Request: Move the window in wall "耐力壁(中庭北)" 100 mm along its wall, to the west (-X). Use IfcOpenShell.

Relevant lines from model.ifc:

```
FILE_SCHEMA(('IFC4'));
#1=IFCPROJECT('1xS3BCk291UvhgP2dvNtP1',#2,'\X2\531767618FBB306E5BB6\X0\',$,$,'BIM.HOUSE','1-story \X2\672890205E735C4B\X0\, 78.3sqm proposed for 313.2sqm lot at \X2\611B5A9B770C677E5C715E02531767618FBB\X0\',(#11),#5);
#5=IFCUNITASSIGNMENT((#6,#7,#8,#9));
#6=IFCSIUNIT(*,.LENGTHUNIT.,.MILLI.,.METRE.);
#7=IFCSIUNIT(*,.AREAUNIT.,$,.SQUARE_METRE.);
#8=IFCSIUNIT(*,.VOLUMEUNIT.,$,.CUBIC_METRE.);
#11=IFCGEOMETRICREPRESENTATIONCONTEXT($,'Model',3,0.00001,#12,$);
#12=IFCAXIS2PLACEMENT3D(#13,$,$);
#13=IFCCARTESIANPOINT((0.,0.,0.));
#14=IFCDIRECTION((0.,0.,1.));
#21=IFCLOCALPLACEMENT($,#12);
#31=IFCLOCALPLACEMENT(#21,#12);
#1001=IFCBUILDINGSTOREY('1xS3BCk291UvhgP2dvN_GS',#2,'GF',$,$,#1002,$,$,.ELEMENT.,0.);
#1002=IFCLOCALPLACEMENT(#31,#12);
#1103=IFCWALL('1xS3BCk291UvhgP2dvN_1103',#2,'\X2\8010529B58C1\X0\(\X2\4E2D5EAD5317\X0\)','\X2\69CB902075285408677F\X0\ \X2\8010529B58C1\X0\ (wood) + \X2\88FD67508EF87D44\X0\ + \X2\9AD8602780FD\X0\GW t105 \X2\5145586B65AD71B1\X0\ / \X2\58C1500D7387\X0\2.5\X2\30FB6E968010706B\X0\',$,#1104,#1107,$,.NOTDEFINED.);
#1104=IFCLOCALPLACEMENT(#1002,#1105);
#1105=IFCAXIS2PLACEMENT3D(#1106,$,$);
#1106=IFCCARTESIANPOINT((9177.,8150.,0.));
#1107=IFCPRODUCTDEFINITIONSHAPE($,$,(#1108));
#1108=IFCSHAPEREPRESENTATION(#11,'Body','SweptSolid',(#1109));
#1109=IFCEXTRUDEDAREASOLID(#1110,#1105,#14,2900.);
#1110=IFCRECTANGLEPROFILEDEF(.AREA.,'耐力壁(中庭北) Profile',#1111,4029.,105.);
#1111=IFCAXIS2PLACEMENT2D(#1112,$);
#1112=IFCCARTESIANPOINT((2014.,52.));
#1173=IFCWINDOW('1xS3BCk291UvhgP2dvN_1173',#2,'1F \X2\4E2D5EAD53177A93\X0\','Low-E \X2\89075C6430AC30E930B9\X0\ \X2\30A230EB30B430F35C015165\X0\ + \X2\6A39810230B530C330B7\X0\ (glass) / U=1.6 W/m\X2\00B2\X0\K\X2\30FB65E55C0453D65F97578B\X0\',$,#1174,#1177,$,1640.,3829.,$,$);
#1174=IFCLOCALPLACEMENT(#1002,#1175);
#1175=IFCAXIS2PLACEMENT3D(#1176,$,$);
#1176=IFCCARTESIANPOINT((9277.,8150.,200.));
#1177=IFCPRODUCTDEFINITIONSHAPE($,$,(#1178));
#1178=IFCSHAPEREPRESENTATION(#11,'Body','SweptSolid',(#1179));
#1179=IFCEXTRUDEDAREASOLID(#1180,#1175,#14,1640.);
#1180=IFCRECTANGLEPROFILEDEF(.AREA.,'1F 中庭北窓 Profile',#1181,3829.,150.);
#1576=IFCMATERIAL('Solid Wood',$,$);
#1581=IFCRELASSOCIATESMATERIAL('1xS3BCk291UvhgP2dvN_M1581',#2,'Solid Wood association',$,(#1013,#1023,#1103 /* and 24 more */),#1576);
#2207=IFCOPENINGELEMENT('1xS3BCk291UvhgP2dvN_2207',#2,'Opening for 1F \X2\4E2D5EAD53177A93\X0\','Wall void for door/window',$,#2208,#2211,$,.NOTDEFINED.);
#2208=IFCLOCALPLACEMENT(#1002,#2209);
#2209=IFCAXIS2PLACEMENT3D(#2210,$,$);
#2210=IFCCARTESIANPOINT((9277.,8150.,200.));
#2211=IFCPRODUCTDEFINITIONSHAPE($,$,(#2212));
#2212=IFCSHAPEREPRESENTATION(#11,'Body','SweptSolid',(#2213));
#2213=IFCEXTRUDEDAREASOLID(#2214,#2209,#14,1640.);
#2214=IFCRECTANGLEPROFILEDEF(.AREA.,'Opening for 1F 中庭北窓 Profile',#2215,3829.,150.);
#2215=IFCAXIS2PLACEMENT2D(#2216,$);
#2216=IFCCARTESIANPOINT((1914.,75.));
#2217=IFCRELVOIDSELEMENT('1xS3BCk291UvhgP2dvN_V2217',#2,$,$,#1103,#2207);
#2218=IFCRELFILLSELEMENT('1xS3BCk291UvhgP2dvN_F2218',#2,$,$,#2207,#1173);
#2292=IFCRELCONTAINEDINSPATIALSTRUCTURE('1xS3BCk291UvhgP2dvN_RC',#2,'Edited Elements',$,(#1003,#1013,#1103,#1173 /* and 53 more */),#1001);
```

```python
import ifcopenshell
import ifcopenshell.api.geometry
import ifcopenshell.util.placement
import ifcopenshell.util.unit

model = ifcopenshell.open("model.ifc")
unit_scale = ifcopenshell.util.unit.calculate_unit_scale(model)

window = model.by_guid("1xS3BCk291UvhgP2dvN_1173")
opening = window.FillsVoids[0].RelatingOpeningElement
wall = opening.VoidsElements[0].RelatingBuildingElement

wall_matrix = ifcopenshell.util.placement.get_local_placement(wall.ObjectPlacement)
shift = wall_matrix[:3, 0] * -0.1 / unit_scale
before = ifcopenshell.util.placement.get_local_placement(window.ObjectPlacement)[:3, 3].copy()

# The window is not placed relative to its opening, so move both.
for product in (opening, window):
    matrix = ifcopenshell.util.placement.get_local_placement(product.ObjectPlacement)
    matrix[:3, 3] += shift
    ifcopenshell.api.geometry.edit_object_placement(model, product=product, matrix=matrix, is_si=False)

after = ifcopenshell.util.placement.get_local_placement(window.ObjectPlacement)[:3, 3]
print("window moved by", (after - before).round(3) + 0.0)

model.write("model_v2.ifc")
```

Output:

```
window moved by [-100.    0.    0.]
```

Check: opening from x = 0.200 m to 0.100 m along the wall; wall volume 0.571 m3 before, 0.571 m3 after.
